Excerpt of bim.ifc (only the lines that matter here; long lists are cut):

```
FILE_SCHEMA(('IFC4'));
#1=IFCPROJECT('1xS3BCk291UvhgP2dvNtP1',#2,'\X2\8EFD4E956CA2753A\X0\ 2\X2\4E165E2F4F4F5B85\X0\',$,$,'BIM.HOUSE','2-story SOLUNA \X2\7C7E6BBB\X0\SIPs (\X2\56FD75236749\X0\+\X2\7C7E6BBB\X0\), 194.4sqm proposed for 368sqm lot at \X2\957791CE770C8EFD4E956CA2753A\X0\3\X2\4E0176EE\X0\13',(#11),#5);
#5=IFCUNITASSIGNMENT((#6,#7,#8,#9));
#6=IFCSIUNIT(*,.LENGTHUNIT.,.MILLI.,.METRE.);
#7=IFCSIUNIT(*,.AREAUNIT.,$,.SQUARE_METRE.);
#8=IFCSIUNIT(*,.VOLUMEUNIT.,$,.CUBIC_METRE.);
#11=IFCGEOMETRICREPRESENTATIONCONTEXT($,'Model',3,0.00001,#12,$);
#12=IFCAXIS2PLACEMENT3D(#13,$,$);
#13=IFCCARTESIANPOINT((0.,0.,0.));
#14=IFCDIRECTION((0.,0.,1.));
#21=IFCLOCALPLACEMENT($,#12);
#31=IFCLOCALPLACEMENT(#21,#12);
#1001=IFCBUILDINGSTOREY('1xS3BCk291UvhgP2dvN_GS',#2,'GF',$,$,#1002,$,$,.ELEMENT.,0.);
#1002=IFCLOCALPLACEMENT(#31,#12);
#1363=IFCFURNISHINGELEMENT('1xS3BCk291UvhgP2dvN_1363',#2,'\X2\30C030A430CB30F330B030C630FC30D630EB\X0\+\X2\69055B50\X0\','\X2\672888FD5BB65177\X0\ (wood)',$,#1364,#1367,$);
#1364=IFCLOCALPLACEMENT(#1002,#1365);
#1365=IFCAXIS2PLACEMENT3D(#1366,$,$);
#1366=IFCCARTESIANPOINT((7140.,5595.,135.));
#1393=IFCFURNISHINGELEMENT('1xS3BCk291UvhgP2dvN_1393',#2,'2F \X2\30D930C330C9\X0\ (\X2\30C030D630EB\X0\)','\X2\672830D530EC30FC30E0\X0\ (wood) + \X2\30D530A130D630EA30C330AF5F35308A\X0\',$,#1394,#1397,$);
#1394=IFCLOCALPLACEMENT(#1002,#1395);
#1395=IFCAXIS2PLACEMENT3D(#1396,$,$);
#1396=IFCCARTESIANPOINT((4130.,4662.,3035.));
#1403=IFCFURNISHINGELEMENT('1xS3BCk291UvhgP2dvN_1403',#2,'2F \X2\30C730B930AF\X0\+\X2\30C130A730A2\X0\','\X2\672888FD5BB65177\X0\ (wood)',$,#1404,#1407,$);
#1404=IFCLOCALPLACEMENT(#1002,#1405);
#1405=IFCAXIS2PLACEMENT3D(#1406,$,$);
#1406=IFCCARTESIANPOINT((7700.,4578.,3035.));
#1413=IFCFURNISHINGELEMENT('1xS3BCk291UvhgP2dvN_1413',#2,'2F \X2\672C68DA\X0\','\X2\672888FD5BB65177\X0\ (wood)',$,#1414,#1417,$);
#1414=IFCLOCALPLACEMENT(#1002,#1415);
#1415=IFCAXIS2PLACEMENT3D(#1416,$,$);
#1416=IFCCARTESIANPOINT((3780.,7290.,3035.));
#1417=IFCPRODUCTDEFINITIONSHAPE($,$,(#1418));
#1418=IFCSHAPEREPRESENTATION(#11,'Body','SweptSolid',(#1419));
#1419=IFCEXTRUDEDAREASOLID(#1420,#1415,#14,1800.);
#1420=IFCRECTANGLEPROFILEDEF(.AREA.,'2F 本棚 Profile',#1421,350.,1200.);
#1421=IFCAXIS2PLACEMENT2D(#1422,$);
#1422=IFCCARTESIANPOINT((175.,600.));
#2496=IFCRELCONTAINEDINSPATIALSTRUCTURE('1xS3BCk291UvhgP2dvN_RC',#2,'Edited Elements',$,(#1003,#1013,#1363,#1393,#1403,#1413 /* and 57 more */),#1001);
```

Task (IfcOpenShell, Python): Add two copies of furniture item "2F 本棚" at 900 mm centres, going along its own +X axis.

```python
import ifcopenshell
import ifcopenshell.api.geometry
import ifcopenshell.api.root
import ifcopenshell.util.element
import ifcopenshell.util.placement
import ifcopenshell.util.unit

model = ifcopenshell.open("bim.ifc")
unit_scale = ifcopenshell.util.unit.calculate_unit_scale(model)


def reuse_history(source, copy):
    """copy_class also copies each property set's owner history, people and application; keep the originals."""
    for rel in copy.IsDefinedBy:
        if rel.is_a("IfcRelDefinesByProperties") and (history := rel.RelatingPropertyDefinition.OwnerHistory):
            rel.RelatingPropertyDefinition.OwnerHistory = source.OwnerHistory
            ifcopenshell.util.element.remove_deep2(model, history)


source = model.by_guid("1xS3BCk291UvhgP2dvN_1413")
base = ifcopenshell.util.placement.get_local_placement(source.ObjectPlacement)
step = base[:3, 0] * 0.9 / unit_scale

for i in range(1, 3):
    copy = ifcopenshell.api.root.copy_class(model, product=source)
    copy.Representation = ifcopenshell.util.element.copy_deep(
        model, source.Representation, exclude=["IfcGeometricRepresentationContext", "IfcRepresentationMap"]
    )
    reuse_history(source, copy)
    matrix = base.copy()
    matrix[:3, 3] += i * step
    print("added at", matrix[:3, 3].round(3) + 0.0)
    ifcopenshell.api.geometry.edit_object_placement(model, product=copy, matrix=matrix, is_si=False)

model.write("bim-out.ifc")
```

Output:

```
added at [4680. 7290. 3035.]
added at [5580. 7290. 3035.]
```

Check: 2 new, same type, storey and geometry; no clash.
